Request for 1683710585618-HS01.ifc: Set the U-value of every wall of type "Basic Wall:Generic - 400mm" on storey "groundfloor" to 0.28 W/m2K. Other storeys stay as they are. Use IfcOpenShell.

First a look at what the model holds.

```python
import ifcopenshell
import ifcopenshell.util.element

model = ifcopenshell.open("1683710585618-HS01.ifc")
print(model.schema)
storey = next(s for s in model.by_type("IfcBuildingStorey") if s.Name == "groundfloor")
walls = [e for e in ifcopenshell.util.element.get_decomposition(storey) if e.is_a("IfcWall")]
seen = {}
for e in walls:
    element_type = ifcopenshell.util.element.get_type(e)
    key = (element_type.Name if element_type != e and element_type else None, ifcopenshell.util.element.get_pset(e, "Pset_WallCommon", "ThermalTransmittance"))
    seen[key] = seen.get(key, 0) + 1
for (name, value), count in sorted(seen.items(), key=str):
    print(count, "x", name, "|", value)
```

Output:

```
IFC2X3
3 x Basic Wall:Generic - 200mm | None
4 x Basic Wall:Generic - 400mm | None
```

```python
import ifcopenshell
import ifcopenshell.api.pset
import ifcopenshell.util.element

model = ifcopenshell.open("1683710585618-HS01.ifc")

storey = next(s for s in model.by_type("IfcBuildingStorey") if s.Name == "groundfloor")
walls = [e for e in ifcopenshell.util.element.get_decomposition(storey) if e.is_a("IfcWall")]

count = 0
for e in walls:
    element_type = ifcopenshell.util.element.get_type(e)
    if element_type in (None, e) or element_type.Name != "Basic Wall:Generic - 400mm":
        continue
    # add_pset returns the element's existing set when there is one.
    pset = ifcopenshell.api.pset.add_pset(model, product=e, name="Pset_WallCommon")
    ifcopenshell.api.pset.edit_pset(model, pset=pset, properties={"ThermalTransmittance": 0.28})
    count += 1

print(count, "walls updated")

model.write("1683710585618-HS01_edited.ifc")
```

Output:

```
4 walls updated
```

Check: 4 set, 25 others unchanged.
